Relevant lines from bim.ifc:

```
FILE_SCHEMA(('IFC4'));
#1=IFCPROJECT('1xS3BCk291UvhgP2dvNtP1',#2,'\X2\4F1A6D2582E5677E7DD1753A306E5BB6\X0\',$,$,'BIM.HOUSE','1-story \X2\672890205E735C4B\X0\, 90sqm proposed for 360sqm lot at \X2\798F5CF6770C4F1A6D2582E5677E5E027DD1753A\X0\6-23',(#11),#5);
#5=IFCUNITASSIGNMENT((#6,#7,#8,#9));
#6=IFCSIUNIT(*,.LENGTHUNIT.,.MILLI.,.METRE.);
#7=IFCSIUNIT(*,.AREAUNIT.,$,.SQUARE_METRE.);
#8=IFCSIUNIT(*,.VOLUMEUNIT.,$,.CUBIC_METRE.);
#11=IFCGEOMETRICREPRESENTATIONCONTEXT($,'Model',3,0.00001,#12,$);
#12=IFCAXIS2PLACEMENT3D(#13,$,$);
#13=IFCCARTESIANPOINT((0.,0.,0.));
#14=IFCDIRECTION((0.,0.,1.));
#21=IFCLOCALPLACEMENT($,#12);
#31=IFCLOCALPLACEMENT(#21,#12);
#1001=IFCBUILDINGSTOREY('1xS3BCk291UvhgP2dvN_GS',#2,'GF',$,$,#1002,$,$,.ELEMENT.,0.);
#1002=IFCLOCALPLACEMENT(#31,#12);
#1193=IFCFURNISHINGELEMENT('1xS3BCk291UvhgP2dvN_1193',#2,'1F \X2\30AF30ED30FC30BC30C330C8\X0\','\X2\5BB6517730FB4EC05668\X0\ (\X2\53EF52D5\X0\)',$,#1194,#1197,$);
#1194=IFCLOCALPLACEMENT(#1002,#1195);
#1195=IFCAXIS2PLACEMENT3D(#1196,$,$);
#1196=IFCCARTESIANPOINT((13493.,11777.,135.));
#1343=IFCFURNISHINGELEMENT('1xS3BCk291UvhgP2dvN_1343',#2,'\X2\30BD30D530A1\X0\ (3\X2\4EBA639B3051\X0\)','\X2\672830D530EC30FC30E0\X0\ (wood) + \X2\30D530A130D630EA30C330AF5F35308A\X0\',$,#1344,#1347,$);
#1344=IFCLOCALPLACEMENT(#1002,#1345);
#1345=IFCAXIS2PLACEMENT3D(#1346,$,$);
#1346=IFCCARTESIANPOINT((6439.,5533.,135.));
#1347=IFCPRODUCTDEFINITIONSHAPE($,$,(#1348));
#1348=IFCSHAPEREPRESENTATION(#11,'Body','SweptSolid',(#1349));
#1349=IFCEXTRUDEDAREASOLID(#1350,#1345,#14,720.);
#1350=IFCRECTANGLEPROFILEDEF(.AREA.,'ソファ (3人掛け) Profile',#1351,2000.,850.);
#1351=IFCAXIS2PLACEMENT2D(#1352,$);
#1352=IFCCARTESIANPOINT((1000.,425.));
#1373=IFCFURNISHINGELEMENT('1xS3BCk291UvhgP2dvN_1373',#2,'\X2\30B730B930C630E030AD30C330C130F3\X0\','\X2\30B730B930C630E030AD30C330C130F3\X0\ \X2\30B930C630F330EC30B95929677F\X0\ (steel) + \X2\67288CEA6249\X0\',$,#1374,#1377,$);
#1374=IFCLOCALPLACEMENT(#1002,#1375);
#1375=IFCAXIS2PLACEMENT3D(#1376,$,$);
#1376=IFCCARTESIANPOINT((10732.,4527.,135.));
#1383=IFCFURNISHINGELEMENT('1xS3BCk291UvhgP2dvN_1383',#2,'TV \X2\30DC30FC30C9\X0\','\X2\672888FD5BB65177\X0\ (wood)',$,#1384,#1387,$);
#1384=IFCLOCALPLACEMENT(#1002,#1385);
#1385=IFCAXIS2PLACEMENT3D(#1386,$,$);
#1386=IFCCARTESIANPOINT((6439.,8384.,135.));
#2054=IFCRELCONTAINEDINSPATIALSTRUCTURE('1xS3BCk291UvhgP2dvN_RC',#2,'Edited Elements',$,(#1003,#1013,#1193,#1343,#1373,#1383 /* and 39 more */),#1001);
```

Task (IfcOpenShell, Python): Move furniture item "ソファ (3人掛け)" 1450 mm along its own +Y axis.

```python
import ifcopenshell
import ifcopenshell.api.geometry
import ifcopenshell.util.placement
import ifcopenshell.util.unit

model = ifcopenshell.open("bim.ifc")
unit_scale = ifcopenshell.util.unit.calculate_unit_scale(model)

item = model.by_guid("1xS3BCk291UvhgP2dvN_1343")
matrix = ifcopenshell.util.placement.get_local_placement(item.ObjectPlacement)
matrix[:3, 3] += matrix[:3, 1] * 1.45 / unit_scale
ifcopenshell.api.geometry.edit_object_placement(model, product=item, matrix=matrix, is_si=False)

print(ifcopenshell.util.placement.get_local_placement(item.ObjectPlacement).round(3) + 0.0)

model.write("bim_updated.ifc")
```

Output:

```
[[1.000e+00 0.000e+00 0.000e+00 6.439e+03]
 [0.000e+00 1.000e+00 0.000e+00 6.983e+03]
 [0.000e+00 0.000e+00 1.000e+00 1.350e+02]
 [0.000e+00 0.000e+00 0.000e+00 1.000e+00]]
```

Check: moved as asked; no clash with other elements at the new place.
